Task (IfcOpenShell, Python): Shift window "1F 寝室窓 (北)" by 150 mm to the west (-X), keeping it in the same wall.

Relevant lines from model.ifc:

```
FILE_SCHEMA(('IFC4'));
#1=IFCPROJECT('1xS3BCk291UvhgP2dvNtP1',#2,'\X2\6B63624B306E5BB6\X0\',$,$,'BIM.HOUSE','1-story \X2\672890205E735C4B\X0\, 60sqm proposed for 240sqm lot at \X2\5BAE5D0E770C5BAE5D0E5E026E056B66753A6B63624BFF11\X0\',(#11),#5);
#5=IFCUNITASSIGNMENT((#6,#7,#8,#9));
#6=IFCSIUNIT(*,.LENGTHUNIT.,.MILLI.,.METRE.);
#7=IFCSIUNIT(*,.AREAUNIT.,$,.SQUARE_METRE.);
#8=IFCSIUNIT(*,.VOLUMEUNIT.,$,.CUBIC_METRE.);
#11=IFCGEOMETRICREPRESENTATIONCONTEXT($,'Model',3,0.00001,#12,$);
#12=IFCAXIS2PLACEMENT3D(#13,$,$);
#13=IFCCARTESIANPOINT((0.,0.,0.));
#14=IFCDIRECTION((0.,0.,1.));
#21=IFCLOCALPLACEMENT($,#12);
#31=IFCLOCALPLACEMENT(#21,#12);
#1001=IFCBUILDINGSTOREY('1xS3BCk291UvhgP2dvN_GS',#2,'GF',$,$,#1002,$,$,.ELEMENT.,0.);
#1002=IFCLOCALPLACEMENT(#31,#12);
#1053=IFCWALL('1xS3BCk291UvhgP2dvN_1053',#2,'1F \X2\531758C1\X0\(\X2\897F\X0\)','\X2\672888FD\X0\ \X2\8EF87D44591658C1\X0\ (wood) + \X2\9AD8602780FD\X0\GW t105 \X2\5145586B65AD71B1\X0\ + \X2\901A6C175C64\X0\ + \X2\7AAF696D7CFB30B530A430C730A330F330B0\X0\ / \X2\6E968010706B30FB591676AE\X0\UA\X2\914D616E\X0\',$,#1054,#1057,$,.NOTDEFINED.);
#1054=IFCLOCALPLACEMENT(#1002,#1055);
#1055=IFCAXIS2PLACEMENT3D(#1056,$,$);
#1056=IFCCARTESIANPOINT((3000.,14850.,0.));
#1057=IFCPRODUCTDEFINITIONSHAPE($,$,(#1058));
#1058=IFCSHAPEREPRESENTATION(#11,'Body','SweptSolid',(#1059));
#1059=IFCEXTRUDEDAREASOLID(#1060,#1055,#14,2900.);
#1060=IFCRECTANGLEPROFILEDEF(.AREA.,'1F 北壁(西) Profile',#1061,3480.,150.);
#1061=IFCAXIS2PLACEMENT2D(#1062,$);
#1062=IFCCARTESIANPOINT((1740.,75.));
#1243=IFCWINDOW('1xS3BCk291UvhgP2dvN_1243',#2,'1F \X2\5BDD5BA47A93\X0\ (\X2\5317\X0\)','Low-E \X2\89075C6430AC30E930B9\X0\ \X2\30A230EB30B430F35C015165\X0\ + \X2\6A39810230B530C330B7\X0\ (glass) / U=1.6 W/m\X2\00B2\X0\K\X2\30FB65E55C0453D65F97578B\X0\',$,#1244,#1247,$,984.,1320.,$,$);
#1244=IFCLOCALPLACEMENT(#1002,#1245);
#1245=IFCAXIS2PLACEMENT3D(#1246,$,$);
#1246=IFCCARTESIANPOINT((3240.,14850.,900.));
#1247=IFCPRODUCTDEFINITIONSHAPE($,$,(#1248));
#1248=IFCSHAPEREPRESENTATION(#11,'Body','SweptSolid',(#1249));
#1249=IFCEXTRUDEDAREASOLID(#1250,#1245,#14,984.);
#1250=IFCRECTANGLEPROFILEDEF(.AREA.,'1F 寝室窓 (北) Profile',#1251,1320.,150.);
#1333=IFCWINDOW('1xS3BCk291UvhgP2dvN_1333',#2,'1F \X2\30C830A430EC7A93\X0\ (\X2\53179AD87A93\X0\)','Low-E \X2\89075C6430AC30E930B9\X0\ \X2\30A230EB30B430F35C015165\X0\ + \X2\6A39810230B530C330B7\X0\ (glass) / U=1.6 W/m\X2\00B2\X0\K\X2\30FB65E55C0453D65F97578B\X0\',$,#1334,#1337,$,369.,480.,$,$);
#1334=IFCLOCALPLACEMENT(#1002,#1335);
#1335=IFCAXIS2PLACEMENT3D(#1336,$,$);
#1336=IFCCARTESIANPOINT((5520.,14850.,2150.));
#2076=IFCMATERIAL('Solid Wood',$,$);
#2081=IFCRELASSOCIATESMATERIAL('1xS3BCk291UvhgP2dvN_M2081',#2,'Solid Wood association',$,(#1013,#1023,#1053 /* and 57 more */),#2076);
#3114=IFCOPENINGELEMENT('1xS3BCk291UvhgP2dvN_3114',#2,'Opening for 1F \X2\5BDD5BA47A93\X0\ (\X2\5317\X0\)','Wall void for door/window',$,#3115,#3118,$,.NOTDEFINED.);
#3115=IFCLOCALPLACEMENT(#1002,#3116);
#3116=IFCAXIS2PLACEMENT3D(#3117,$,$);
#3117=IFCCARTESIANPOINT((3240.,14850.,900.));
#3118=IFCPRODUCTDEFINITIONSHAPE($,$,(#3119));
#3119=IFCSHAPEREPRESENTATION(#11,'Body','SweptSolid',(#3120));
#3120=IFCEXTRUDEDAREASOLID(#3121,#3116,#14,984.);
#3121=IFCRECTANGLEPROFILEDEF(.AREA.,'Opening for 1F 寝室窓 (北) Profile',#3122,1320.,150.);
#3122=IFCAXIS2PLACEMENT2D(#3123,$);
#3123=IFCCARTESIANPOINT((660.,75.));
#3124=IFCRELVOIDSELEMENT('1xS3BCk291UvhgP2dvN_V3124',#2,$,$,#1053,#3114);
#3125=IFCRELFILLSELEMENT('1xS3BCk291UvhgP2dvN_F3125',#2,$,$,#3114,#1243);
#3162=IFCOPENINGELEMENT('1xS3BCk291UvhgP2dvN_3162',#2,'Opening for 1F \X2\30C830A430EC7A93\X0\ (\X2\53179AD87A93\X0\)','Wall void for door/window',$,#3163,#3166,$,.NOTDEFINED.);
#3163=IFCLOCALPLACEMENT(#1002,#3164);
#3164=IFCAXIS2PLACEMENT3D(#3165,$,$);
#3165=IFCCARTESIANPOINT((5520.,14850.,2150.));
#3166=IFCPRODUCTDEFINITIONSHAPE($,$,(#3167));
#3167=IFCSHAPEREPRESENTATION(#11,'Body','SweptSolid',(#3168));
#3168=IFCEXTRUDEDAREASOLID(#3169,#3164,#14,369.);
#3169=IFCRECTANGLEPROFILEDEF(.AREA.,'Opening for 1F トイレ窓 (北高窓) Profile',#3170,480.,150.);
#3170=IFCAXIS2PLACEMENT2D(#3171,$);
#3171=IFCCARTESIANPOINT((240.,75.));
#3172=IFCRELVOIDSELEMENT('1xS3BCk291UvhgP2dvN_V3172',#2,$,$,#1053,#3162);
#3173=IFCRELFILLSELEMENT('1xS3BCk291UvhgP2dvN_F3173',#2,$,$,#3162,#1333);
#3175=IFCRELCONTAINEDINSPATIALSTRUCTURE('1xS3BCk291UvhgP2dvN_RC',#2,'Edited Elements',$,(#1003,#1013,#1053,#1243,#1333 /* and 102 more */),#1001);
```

```python
import ifcopenshell
import ifcopenshell.api.geometry
import ifcopenshell.util.placement
import ifcopenshell.util.unit

model = ifcopenshell.open("model.ifc")
unit_scale = ifcopenshell.util.unit.calculate_unit_scale(model)

window = model.by_id(1243)
opening = window.FillsVoids[0].RelatingOpeningElement
wall = opening.VoidsElements[0].RelatingBuildingElement

wall_matrix = ifcopenshell.util.placement.get_local_placement(wall.ObjectPlacement)
shift = wall_matrix[:3, 0] * -0.15 / unit_scale
before = ifcopenshell.util.placement.get_local_placement(window.ObjectPlacement)[:3, 3].copy()

# The window is not placed relative to its opening, so move both.
for product in (opening, window):
    matrix = ifcopenshell.util.placement.get_local_placement(product.ObjectPlacement)
    matrix[:3, 3] += shift
    ifcopenshell.api.geometry.edit_object_placement(model, product=product, matrix=matrix, is_si=False)

after = ifcopenshell.util.placement.get_local_placement(window.ObjectPlacement)[:3, 3]
print("window moved by", (after - before).round(3) + 0.0)

model.write("model_v2.ifc")
```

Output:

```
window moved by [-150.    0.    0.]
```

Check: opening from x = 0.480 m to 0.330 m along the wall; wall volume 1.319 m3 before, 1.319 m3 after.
